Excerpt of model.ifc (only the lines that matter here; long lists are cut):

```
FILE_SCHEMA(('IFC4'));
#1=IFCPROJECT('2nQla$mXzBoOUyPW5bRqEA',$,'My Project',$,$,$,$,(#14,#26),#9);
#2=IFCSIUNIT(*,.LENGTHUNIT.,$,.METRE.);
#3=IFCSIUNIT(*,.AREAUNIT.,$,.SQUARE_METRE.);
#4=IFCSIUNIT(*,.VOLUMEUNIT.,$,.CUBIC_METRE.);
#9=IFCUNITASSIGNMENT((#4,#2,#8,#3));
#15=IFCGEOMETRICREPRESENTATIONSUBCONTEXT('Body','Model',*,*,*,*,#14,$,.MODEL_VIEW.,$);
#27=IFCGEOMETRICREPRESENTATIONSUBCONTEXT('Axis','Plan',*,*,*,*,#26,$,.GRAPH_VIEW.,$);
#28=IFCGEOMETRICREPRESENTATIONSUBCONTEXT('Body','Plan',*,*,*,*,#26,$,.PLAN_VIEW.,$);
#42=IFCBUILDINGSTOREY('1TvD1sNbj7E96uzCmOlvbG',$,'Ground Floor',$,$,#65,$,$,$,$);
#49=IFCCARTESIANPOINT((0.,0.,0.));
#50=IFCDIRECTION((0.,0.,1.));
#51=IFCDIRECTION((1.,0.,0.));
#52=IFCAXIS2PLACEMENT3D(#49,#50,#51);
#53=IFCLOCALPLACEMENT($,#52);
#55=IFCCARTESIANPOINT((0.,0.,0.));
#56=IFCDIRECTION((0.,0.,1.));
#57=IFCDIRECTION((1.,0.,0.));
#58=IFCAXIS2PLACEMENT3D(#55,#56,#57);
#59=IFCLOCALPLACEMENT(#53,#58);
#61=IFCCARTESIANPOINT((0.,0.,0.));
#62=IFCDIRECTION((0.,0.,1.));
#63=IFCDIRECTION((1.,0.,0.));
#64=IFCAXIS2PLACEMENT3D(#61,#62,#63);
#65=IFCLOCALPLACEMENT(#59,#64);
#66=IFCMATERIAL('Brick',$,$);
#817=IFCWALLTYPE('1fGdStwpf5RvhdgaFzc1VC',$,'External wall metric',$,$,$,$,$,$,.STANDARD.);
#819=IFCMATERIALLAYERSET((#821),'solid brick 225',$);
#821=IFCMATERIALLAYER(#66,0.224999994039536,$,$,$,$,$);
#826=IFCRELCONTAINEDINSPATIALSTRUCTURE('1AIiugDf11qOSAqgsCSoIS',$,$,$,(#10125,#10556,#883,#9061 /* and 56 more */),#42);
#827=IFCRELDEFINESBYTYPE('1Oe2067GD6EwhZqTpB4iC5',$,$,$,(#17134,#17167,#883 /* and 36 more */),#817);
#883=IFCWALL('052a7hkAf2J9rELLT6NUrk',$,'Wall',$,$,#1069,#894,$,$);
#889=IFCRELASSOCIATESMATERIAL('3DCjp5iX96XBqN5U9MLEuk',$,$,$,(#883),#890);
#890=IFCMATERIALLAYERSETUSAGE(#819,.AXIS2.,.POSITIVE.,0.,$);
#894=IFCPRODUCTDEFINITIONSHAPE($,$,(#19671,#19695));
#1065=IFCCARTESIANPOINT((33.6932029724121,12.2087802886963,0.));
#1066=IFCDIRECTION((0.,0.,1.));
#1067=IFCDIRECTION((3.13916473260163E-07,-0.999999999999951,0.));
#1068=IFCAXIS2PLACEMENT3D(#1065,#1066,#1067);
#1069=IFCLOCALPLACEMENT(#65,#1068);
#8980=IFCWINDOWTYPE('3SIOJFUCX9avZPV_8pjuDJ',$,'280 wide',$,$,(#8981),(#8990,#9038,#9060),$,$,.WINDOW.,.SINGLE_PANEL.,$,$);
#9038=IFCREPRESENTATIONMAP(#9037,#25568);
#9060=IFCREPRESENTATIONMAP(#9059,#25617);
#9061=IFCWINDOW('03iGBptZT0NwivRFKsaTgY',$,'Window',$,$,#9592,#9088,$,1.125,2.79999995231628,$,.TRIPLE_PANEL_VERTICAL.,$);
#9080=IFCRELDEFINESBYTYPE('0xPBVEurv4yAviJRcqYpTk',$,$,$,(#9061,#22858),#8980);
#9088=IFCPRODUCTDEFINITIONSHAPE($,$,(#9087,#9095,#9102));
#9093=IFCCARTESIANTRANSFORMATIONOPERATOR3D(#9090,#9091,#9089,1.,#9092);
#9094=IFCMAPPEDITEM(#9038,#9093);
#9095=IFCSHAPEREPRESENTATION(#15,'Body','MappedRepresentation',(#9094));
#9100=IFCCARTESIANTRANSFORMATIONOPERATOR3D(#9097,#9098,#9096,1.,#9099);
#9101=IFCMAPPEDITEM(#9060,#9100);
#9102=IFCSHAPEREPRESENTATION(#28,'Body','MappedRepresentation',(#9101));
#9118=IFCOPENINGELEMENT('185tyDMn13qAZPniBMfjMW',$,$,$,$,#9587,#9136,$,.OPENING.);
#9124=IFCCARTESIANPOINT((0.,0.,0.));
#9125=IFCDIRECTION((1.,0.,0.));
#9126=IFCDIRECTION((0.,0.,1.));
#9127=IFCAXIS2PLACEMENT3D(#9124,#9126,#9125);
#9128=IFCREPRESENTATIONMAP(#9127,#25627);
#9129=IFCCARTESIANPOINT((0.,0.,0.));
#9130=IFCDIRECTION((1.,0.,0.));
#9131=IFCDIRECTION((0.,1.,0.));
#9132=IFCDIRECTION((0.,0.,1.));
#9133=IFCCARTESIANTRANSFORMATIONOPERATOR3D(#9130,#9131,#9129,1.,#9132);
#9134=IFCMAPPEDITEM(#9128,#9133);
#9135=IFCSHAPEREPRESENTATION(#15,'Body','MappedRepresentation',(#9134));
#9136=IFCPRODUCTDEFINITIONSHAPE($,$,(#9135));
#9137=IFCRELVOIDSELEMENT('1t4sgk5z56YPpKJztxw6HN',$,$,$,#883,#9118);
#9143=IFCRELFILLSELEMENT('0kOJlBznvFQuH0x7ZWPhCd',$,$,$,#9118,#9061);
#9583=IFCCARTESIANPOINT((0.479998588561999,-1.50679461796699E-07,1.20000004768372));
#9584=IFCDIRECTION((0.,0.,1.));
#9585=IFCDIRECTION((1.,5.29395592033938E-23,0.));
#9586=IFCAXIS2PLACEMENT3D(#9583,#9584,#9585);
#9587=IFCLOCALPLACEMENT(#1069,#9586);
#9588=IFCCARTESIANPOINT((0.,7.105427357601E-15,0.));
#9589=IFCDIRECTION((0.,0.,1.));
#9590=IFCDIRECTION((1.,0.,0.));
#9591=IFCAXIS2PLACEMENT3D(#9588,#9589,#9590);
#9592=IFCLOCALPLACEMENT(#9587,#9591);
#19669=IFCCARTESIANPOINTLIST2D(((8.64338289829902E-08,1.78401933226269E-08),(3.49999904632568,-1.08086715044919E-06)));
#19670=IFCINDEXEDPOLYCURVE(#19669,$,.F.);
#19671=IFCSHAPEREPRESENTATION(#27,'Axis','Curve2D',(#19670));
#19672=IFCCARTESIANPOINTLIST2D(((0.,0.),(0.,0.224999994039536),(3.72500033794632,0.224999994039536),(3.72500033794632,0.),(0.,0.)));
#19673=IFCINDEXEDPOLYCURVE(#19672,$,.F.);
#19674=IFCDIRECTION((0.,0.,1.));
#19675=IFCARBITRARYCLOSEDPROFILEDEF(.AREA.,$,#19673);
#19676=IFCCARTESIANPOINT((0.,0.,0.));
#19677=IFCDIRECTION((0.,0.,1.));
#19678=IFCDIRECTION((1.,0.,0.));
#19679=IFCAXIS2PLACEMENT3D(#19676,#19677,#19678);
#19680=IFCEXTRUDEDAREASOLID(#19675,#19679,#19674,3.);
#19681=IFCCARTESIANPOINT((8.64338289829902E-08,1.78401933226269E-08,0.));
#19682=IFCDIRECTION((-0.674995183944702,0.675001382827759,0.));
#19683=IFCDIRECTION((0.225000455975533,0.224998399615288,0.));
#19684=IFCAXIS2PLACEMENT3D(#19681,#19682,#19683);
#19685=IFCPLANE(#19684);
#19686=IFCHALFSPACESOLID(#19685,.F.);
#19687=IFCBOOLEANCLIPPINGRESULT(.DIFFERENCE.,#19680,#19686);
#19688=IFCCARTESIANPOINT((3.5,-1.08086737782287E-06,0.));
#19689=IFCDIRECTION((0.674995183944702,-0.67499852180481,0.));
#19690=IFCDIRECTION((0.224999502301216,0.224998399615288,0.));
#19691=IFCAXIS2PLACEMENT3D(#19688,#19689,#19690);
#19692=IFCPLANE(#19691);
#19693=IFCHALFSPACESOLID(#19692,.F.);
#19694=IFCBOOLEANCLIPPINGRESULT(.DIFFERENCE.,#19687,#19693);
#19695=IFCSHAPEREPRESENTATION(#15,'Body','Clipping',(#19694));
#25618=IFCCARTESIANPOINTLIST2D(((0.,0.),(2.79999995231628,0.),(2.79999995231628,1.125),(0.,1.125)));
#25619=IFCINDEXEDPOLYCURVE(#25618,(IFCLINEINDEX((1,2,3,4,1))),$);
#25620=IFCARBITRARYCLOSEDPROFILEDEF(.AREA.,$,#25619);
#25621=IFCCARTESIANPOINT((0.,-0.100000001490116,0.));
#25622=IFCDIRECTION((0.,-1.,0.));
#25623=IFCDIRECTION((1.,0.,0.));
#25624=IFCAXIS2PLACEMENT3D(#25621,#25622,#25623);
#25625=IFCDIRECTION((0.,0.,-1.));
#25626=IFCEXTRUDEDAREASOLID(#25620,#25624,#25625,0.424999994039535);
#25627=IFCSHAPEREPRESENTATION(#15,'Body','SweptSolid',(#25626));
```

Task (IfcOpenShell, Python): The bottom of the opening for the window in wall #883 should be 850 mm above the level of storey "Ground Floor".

```python
import numpy as np
import ifcopenshell
import ifcopenshell.api.geometry
import ifcopenshell.geom
import ifcopenshell.util.element
import ifcopenshell.util.placement
import ifcopenshell.util.shape
import ifcopenshell.util.unit

model = ifcopenshell.open("model.ifc")
unit_scale = ifcopenshell.util.unit.calculate_unit_scale(model)

window = model.by_guid("03iGBptZT0NwivRFKsaTgY")
opening = window.FillsVoids[0].RelatingOpeningElement
storey = ifcopenshell.util.element.get_container(window, ifc_class="IfcBuildingStorey")
level = ifcopenshell.util.placement.get_local_placement(storey.ObjectPlacement)[2, 3]

# The opening's origin need not be at the sill, so measure its lowest point.
shape = ifcopenshell.geom.create_shape(ifcopenshell.geom.settings(), opening)
bottom = ifcopenshell.util.shape.get_shape_bottom_elevation(shape, shape.geometry) / unit_scale
dz = level + 0.85 - bottom

shift = np.array([0.0, 0.0, dz])
# The window is placed relative to its opening, so it follows when the opening moves.
matrix = ifcopenshell.util.placement.get_local_placement(opening.ObjectPlacement)
matrix[:3, 3] += shift
ifcopenshell.api.geometry.edit_object_placement(
    model, product=opening, matrix=matrix, is_si=False, should_transform_children=True
)

print(f"moved by {dz * unit_scale:+.3f} m")

model.write("model_edited.ifc")
```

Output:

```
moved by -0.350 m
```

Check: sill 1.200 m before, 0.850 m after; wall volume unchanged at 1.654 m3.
